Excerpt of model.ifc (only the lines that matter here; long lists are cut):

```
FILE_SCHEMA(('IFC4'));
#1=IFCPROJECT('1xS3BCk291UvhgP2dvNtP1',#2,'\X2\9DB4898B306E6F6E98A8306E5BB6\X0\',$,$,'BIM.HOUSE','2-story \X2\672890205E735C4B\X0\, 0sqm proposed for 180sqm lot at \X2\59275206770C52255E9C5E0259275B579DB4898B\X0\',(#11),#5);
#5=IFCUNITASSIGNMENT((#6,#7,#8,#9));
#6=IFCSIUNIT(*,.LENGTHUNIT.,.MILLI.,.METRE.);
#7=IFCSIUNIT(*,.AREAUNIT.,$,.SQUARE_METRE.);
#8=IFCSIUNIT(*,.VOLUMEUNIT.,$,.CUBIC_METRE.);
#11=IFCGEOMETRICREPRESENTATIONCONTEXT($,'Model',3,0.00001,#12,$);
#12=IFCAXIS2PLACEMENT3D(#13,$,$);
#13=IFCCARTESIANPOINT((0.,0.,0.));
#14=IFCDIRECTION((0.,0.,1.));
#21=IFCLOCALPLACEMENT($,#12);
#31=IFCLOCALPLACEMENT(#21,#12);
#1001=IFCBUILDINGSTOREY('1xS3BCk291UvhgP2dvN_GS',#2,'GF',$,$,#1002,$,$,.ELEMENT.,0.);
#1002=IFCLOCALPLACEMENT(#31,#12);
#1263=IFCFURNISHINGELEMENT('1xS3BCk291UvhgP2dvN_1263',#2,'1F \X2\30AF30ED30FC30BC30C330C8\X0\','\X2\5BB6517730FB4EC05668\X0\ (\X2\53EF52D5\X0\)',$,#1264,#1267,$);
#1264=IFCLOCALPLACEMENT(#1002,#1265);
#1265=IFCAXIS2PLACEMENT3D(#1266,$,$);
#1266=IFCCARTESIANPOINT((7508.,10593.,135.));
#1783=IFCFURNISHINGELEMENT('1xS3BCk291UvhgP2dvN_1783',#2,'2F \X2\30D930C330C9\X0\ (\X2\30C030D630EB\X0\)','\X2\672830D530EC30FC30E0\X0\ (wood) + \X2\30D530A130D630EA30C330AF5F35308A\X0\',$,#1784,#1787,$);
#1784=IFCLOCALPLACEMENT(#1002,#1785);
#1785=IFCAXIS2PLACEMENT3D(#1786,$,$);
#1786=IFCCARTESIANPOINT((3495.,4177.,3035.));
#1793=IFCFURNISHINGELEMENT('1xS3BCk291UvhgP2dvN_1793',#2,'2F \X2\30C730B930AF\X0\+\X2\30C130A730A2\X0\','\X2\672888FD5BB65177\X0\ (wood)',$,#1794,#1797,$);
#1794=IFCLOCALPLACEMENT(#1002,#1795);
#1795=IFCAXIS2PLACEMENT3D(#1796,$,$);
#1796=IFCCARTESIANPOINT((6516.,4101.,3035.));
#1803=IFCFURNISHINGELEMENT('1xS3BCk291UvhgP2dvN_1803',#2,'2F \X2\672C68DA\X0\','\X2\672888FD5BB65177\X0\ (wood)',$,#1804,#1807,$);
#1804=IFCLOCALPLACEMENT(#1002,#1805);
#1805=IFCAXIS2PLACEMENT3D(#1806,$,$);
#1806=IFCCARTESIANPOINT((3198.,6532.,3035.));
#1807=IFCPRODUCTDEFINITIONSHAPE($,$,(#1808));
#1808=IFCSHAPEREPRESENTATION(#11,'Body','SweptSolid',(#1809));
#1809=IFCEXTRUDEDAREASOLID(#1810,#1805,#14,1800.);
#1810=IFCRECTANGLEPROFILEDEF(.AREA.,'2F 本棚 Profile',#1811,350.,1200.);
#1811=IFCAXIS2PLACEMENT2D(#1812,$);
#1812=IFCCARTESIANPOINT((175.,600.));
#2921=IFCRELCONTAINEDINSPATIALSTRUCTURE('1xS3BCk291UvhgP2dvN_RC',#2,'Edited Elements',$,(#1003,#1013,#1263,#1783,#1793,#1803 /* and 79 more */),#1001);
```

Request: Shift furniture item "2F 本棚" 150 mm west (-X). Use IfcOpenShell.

```python
import ifcopenshell
import ifcopenshell.api.geometry
import ifcopenshell.util.placement
import ifcopenshell.util.unit

model = ifcopenshell.open("model.ifc")
unit_scale = ifcopenshell.util.unit.calculate_unit_scale(model)

item = model.by_guid("1xS3BCk291UvhgP2dvN_1803")
matrix = ifcopenshell.util.placement.get_local_placement(item.ObjectPlacement)
matrix[0, 3] -= 0.15 / unit_scale
ifcopenshell.api.geometry.edit_object_placement(model, product=item, matrix=matrix, is_si=False)

print(ifcopenshell.util.placement.get_local_placement(item.ObjectPlacement).round(3) + 0.0)

model.write("model_edited.ifc")
```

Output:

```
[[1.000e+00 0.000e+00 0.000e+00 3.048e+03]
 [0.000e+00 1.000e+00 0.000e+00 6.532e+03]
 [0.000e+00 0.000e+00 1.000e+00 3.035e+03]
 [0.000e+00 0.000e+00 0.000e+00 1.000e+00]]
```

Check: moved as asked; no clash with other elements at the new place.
